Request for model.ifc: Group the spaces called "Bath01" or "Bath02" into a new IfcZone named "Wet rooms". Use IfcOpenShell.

First a look at what the model holds.

```python
import ifcopenshell

model = ifcopenshell.open("model.ifc")
print(model.schema)
seen = {}
for space in model.by_type("IfcSpace"):
    seen[space.Name] = seen.get(space.Name, 0) + 1
for name, count in sorted(seen.items(), key=str):
    print(count, "x", name)
print("zones:", [z.Name for z in model.by_type("IfcZone")][:20])
```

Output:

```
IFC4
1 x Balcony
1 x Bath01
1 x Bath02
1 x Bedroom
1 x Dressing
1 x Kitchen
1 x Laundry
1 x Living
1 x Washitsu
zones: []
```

```python
import ifcopenshell
import ifcopenshell.api.group
import ifcopenshell.api.root

model = ifcopenshell.open("model.ifc")

names = {"Bath01", "Bath02"}
spaces = [s for s in model.by_type("IfcSpace") if s.Name in names]

zone = ifcopenshell.api.root.create_entity(model, ifc_class="IfcZone", name="Wet rooms")
ifcopenshell.api.group.assign_group(model, products=spaces, group=zone)
print(len(spaces), "spaces in", zone.Name)

model.write("model_updated.ifc")
```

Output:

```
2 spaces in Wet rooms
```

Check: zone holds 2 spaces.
